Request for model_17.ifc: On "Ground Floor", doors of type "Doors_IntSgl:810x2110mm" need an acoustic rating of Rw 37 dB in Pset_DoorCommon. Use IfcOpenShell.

First a look at what the model holds.

```python
import ifcopenshell
import ifcopenshell.util.element

model = ifcopenshell.open("model_17.ifc")
print(model.schema)
storey = next(s for s in model.by_type("IfcBuildingStorey") if s.Name == "Ground Floor")
doors = [e for e in ifcopenshell.util.element.get_decomposition(storey) if e.is_a("IfcDoor")]
seen = {}
for e in doors:
    element_type = ifcopenshell.util.element.get_type(e)
    key = (element_type.Name if element_type != e and element_type else None, ifcopenshell.util.element.get_pset(e, "Pset_DoorCommon", "AcousticRating"))
    seen[key] = seen.get(key, 0) + 1
for (name, value), count in sorted(seen.items(), key=str):
    print(count, "x", name, "|", value)
```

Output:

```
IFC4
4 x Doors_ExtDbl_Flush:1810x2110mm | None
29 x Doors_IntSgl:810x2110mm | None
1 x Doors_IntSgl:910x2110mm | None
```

```python
import ifcopenshell
import ifcopenshell.api.pset
import ifcopenshell.util.element

model = ifcopenshell.open("model_17.ifc")

storey = next(s for s in model.by_type("IfcBuildingStorey") if s.Name == "Ground Floor")
doors = [e for e in ifcopenshell.util.element.get_decomposition(storey) if e.is_a("IfcDoor")]

count = 0
for e in doors:
    element_type = ifcopenshell.util.element.get_type(e)
    if element_type in (None, e) or element_type.Name != "Doors_IntSgl:810x2110mm":
        continue
    # add_pset returns the element's existing set when there is one.
    pset = ifcopenshell.api.pset.add_pset(model, product=e, name="Pset_DoorCommon")
    ifcopenshell.api.pset.edit_pset(model, pset=pset, properties={"AcousticRating": "Rw 37 dB"})
    count += 1

print(count, "doors updated")

model.write("model_17-out.ifc")
```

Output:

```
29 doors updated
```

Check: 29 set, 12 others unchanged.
